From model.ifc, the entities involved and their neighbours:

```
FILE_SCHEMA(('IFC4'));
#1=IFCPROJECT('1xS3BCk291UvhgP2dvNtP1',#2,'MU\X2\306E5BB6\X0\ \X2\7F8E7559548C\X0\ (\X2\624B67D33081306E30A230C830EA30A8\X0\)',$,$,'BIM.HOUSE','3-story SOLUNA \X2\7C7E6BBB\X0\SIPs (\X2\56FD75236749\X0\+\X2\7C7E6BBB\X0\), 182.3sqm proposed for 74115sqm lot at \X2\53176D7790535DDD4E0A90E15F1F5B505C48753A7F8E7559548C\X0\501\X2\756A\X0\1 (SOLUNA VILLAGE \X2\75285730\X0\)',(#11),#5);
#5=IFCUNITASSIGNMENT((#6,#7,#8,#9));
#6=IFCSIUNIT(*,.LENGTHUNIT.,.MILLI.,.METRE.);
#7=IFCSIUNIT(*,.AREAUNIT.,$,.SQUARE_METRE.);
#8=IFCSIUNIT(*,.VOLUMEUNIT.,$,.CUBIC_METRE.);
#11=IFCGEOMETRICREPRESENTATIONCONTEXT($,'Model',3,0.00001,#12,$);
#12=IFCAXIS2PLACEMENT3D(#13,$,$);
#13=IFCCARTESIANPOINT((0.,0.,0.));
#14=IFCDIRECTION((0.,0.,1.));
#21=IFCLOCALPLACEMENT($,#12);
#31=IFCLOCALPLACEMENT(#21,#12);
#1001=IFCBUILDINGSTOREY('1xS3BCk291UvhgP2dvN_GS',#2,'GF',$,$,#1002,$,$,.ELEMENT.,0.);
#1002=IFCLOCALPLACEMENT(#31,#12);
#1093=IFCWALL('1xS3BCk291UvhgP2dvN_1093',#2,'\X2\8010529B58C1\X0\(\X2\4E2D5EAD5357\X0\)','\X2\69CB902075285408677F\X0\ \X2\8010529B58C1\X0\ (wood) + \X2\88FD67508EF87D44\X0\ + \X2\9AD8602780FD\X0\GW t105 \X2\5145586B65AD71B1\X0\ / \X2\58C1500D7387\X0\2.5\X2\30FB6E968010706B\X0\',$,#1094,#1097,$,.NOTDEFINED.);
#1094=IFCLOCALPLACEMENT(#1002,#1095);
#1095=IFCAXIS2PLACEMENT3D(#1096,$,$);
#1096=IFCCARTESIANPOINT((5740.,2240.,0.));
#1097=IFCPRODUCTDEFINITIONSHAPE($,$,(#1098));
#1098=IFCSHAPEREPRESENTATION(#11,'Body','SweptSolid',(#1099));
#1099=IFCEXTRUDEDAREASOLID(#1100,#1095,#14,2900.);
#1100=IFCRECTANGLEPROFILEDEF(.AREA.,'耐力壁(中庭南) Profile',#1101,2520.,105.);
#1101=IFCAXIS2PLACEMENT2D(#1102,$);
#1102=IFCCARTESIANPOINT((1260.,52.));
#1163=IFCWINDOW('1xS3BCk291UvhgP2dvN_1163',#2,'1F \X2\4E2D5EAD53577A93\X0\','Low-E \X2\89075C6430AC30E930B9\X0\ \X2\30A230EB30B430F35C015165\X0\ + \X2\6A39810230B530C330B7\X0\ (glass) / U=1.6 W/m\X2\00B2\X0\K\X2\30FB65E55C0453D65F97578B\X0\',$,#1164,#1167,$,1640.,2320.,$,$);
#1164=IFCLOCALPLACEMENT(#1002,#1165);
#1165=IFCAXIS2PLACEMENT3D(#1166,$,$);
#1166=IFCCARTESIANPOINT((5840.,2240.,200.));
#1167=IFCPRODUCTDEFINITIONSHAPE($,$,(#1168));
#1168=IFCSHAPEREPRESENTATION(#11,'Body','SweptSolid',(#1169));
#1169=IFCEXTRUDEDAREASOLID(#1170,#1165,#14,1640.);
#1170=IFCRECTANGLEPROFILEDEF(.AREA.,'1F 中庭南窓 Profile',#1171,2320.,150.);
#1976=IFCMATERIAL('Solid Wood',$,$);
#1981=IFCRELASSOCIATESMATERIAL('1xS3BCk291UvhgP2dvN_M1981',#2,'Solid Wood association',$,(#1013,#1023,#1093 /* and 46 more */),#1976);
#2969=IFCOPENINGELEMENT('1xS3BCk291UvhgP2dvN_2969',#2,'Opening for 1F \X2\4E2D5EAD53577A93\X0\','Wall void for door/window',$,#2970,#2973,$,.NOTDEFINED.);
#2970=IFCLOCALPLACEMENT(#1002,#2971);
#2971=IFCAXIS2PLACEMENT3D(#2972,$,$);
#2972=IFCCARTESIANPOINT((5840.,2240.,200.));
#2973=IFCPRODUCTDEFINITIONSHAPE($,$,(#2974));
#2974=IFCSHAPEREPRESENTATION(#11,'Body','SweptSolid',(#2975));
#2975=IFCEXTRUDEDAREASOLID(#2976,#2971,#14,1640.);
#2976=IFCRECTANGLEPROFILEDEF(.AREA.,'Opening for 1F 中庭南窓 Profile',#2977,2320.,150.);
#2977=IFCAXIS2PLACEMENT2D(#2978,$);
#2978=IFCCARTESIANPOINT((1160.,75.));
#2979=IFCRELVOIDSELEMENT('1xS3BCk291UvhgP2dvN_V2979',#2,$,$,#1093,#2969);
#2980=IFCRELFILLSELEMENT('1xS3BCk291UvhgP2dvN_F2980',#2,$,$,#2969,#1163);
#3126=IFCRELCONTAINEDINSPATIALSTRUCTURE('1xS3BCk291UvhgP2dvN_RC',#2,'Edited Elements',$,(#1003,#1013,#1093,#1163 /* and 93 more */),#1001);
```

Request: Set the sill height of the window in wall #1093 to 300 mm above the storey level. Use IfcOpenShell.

```python
import numpy as np
import ifcopenshell
import ifcopenshell.api.geometry
import ifcopenshell.geom
import ifcopenshell.util.element
import ifcopenshell.util.placement
import ifcopenshell.util.shape
import ifcopenshell.util.unit

model = ifcopenshell.open("model.ifc")
unit_scale = ifcopenshell.util.unit.calculate_unit_scale(model)

window = model.by_id(1163)
opening = window.FillsVoids[0].RelatingOpeningElement
storey = ifcopenshell.util.element.get_container(window, ifc_class="IfcBuildingStorey")
level = ifcopenshell.util.placement.get_local_placement(storey.ObjectPlacement)[2, 3]

# The opening's origin need not be at the sill, so measure its lowest point.
shape = ifcopenshell.geom.create_shape(ifcopenshell.geom.settings(), opening)
bottom = ifcopenshell.util.shape.get_shape_bottom_elevation(shape, shape.geometry) / unit_scale
dz = level + 300.0 - bottom

shift = np.array([0.0, 0.0, dz])
# The window is not placed relative to its opening, so move both.
for product in (opening, window):
    matrix = ifcopenshell.util.placement.get_local_placement(product.ObjectPlacement)
    matrix[:3, 3] += shift
    ifcopenshell.api.geometry.edit_object_placement(model, product=product, matrix=matrix, is_si=False)

print(f"moved by {dz * unit_scale:+.3f} m")

model.write("model_edited.ifc")
```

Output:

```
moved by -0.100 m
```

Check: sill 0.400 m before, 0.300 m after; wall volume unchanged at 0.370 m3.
